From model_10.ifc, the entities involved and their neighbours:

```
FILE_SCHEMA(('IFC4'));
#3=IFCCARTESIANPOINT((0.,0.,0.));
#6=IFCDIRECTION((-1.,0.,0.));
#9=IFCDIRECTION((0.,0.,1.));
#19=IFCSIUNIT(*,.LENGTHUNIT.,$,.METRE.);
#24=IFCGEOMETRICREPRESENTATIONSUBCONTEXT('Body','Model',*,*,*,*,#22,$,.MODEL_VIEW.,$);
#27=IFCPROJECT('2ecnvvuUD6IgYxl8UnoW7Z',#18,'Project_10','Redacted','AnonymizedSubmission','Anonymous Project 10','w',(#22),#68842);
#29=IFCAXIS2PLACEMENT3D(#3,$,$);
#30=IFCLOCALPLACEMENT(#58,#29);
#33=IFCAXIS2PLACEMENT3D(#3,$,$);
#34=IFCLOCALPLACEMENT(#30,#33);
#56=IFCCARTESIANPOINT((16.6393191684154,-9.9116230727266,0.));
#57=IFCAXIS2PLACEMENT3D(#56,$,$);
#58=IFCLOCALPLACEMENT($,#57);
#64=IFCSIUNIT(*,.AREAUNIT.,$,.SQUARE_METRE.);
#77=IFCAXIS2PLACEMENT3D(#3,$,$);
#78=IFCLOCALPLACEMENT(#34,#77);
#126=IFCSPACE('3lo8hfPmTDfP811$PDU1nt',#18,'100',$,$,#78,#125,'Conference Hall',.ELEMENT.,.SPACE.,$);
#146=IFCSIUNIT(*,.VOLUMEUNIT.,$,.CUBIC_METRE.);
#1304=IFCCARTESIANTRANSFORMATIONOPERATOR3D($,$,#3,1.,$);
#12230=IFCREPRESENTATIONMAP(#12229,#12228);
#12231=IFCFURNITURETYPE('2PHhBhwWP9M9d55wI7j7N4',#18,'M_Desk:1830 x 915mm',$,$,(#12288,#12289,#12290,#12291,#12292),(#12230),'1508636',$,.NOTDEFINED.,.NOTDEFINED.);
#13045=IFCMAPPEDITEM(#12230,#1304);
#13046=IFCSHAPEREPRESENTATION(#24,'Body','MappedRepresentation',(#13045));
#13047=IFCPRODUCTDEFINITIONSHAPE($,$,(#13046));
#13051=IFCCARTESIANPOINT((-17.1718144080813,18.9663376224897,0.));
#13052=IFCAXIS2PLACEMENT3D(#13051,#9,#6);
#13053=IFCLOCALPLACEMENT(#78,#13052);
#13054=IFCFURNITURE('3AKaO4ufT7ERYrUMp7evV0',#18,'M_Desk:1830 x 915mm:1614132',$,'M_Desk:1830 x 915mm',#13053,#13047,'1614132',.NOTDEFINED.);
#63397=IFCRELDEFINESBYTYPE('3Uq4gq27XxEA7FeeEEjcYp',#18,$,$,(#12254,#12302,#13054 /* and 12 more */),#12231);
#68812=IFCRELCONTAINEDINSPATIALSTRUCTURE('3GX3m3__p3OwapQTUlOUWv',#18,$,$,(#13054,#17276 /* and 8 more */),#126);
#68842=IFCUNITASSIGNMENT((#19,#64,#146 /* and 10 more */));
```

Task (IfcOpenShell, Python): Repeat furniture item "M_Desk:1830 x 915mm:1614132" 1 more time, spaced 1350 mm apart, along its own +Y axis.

```python
import ifcopenshell
import ifcopenshell.api.geometry
import ifcopenshell.api.root
import ifcopenshell.util.element
import ifcopenshell.util.placement
import ifcopenshell.util.unit

model = ifcopenshell.open("model_10.ifc")
unit_scale = ifcopenshell.util.unit.calculate_unit_scale(model)


def reuse_history(source, copy):
    """copy_class also copies each property set's owner history, people and application; keep the originals."""
    for rel in copy.IsDefinedBy:
        if rel.is_a("IfcRelDefinesByProperties") and (history := rel.RelatingPropertyDefinition.OwnerHistory):
            rel.RelatingPropertyDefinition.OwnerHistory = source.OwnerHistory
            ifcopenshell.util.element.remove_deep2(model, history)


source = model.by_guid("3AKaO4ufT7ERYrUMp7evV0")
base = ifcopenshell.util.placement.get_local_placement(source.ObjectPlacement)
step = base[:3, 1] * 1.35 / unit_scale

for i in range(1, 2):
    copy = ifcopenshell.api.root.copy_class(model, product=source)
    copy.Representation = ifcopenshell.util.element.copy_deep(
        model, source.Representation, exclude=["IfcGeometricRepresentationContext", "IfcRepresentationMap"]
    )
    copy.Name = "M_Desk:1830 x 915mm"
    copy.Tag = None
    reuse_history(source, copy)
    matrix = base.copy()
    matrix[:3, 3] += i * step
    print("added at", matrix[:3, 3].round(3) + 0.0)
    ifcopenshell.api.geometry.edit_object_placement(model, product=copy, matrix=matrix, is_si=False)

model.write("model_10_rev.ifc")
```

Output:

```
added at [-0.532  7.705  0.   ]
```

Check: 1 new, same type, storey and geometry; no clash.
